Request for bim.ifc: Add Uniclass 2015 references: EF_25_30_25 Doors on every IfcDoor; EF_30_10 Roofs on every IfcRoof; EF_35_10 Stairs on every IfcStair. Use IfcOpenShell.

First a look at what the model holds.

```python
import ifcopenshell

model = ifcopenshell.open("bim.ifc")
print(model.schema)
print("classifications:", [c.Name for c in model.by_type("IfcClassification")])
for ifc_class in ("IfcDoor", "IfcRoof", "IfcStair", "IfcWall", "IfcWindow"):
    print(ifc_class, len(model.by_type(ifc_class)))
```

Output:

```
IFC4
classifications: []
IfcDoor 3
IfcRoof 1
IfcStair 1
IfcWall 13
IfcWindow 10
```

```python
import ifcopenshell
import ifcopenshell.api.classification

model = ifcopenshell.open("bim.ifc")

system = ifcopenshell.api.classification.add_classification(model, classification="Uniclass 2015")

codes = {
    "IfcDoor": ("EF_25_30_25", "Doors"),
    "IfcRoof": ("EF_30_10", "Roofs"),
    "IfcStair": ("EF_35_10", "Stairs"),
}
for ifc_class, (code, name) in codes.items():
    products = model.by_type(ifc_class)
    ifcopenshell.api.classification.add_reference(
        model, products=products, classification=system, identification=code, name=name
    )
    print(code, len(products))

model.write("bim-out.ifc")
```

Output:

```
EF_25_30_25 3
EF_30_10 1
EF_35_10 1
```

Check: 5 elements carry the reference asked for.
